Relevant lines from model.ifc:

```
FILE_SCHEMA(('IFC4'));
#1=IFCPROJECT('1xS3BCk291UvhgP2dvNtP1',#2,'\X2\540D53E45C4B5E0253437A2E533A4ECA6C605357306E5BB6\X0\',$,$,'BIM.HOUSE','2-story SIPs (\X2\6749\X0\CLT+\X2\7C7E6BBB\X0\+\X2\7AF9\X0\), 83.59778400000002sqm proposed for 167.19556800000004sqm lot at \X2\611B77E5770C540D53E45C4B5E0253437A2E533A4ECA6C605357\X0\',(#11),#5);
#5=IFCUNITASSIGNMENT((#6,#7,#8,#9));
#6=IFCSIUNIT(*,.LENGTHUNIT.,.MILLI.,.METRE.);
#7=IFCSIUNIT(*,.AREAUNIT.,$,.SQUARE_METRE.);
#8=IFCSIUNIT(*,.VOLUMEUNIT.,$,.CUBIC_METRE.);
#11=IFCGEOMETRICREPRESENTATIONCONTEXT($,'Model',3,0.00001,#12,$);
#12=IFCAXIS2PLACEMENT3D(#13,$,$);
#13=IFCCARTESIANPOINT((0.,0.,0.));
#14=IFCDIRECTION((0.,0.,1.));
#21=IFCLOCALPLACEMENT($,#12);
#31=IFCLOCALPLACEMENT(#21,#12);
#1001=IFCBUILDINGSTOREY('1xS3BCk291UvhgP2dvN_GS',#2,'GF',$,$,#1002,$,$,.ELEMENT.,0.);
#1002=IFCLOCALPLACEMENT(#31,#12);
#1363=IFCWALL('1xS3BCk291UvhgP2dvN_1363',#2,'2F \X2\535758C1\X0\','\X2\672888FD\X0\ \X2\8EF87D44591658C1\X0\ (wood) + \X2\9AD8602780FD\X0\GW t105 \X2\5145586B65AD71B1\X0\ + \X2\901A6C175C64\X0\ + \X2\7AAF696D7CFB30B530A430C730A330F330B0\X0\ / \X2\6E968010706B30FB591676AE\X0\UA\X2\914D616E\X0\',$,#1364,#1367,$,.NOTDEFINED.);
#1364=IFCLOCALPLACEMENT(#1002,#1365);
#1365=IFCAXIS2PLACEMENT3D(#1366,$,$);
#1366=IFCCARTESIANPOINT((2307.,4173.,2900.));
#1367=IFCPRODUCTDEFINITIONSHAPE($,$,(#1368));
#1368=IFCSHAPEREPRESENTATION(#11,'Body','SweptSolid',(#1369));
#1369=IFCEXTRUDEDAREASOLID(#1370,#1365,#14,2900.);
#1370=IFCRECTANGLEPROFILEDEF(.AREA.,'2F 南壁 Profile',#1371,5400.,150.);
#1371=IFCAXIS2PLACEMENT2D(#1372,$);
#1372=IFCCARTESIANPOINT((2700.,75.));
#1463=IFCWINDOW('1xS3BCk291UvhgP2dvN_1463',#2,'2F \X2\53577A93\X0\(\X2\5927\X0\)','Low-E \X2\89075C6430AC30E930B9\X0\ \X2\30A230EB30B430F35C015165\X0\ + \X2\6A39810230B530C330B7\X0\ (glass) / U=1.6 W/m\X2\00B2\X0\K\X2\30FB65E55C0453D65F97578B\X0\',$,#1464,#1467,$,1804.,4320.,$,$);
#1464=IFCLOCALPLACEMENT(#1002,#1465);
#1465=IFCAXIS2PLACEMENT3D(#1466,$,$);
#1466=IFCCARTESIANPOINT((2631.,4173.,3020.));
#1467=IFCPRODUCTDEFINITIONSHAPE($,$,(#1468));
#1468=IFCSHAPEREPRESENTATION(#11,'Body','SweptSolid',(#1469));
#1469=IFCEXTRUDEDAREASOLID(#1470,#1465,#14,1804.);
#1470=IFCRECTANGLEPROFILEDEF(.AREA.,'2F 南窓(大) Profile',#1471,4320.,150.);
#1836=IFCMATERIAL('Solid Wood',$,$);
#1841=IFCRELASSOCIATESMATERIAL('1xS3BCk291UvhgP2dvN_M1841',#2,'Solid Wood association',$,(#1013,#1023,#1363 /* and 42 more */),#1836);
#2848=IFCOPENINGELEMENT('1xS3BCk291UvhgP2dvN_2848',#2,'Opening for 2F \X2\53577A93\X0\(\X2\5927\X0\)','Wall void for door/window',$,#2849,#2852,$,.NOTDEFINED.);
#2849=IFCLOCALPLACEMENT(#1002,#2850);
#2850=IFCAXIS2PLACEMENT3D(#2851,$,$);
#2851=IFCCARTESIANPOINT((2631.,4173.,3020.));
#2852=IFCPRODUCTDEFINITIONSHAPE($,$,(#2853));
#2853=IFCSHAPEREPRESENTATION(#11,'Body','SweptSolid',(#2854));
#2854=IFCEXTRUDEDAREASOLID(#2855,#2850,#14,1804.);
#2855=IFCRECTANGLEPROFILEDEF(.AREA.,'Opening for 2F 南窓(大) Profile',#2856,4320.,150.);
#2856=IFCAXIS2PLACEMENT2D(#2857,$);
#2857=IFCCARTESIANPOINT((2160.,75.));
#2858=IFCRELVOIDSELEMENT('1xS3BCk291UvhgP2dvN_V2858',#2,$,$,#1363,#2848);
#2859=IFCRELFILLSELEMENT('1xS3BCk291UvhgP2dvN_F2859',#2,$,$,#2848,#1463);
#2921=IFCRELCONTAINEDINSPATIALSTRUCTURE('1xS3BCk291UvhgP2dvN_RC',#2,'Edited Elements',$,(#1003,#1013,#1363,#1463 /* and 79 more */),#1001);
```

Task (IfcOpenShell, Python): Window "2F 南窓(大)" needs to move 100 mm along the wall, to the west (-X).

```python
import ifcopenshell
import ifcopenshell.api.geometry
import ifcopenshell.util.placement

model = ifcopenshell.open("model.ifc")

window = model.by_id(1463)
opening = window.FillsVoids[0].RelatingOpeningElement
wall = opening.VoidsElements[0].RelatingBuildingElement

wall_matrix = ifcopenshell.util.placement.get_local_placement(wall.ObjectPlacement)
shift = wall_matrix[:3, 0] * -100.0
before = ifcopenshell.util.placement.get_local_placement(window.ObjectPlacement)[:3, 3].copy()

# The window is not placed relative to its opening, so move both.
for product in (opening, window):
    matrix = ifcopenshell.util.placement.get_local_placement(product.ObjectPlacement)
    matrix[:3, 3] += shift
    ifcopenshell.api.geometry.edit_object_placement(model, product=product, matrix=matrix, is_si=False)

after = ifcopenshell.util.placement.get_local_placement(window.ObjectPlacement)[:3, 3]
print("window moved by", (after - before).round(3) + 0.0)

model.write("model_rev.ifc")
```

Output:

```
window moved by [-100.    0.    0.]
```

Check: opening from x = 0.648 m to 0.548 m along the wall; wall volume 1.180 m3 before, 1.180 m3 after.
